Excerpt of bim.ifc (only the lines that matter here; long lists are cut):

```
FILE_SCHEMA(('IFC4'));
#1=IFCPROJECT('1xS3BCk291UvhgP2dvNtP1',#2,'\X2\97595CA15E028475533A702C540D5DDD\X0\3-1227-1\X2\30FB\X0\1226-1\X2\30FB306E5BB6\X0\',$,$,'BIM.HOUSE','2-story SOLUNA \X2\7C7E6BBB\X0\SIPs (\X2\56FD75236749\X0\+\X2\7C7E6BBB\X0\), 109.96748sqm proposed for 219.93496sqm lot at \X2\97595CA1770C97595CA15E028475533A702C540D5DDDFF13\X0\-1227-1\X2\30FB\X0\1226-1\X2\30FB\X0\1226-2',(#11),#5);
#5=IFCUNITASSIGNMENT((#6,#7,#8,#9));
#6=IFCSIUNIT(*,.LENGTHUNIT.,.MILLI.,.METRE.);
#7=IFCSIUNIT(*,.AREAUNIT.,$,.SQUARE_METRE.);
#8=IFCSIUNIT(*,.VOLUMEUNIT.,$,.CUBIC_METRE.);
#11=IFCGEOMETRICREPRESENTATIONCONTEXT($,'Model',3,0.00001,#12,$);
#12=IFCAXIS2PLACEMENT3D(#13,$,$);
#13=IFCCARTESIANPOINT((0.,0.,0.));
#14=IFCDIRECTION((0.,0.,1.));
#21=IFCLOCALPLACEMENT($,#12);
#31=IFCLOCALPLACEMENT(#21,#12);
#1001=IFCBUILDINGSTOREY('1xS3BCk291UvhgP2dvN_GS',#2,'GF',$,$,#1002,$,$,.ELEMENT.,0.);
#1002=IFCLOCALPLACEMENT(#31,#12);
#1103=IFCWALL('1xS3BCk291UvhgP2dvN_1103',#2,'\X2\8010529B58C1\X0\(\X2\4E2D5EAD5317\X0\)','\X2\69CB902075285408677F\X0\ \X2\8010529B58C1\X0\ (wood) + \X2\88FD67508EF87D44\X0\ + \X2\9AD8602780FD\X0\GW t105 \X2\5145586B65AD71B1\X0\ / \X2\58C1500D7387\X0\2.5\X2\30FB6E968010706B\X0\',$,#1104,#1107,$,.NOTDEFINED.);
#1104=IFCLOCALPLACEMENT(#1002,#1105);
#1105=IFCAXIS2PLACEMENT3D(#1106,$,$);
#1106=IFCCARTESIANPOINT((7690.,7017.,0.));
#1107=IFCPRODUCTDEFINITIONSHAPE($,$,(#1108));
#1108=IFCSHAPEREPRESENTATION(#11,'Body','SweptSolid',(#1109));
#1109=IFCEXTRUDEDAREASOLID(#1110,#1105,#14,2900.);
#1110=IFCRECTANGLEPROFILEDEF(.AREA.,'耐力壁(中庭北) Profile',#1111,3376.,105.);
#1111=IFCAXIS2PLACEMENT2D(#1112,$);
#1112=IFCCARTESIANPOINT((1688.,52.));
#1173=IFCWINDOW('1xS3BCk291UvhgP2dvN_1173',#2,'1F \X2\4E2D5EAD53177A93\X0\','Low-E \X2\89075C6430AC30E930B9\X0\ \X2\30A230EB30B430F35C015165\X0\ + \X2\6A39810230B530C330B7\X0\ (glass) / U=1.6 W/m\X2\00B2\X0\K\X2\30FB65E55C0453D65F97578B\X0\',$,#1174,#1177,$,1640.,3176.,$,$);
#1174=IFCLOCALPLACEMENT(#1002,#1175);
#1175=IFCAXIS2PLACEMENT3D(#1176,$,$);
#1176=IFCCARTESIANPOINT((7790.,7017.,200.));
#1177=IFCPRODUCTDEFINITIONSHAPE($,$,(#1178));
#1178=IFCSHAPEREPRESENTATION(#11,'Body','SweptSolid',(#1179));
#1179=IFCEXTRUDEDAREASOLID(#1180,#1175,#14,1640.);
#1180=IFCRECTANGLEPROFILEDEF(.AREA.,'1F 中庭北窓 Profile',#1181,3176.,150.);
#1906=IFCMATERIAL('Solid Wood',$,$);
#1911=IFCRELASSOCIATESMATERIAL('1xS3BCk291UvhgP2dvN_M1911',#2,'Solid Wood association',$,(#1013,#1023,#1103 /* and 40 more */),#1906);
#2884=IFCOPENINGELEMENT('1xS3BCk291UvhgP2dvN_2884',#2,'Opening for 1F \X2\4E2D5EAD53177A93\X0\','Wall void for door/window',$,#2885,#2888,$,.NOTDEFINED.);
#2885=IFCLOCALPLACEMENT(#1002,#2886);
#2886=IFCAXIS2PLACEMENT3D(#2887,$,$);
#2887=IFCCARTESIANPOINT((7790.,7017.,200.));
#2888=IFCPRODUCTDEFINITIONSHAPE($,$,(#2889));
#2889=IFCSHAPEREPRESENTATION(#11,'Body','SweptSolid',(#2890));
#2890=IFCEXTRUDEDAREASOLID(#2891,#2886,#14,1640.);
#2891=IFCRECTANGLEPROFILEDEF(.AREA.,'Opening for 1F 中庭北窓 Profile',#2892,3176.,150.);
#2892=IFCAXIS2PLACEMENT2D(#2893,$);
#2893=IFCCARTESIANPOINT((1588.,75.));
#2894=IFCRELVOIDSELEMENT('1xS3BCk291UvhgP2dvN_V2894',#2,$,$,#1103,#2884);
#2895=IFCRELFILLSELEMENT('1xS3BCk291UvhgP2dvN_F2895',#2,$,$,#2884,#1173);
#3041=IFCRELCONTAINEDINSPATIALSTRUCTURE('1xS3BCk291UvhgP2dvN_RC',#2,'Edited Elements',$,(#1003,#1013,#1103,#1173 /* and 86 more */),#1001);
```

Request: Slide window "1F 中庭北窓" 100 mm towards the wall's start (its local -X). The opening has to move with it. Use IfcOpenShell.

```python
import ifcopenshell
import ifcopenshell.api.geometry
import ifcopenshell.util.placement

model = ifcopenshell.open("bim.ifc")

window = model.by_guid("1xS3BCk291UvhgP2dvN_1173")
opening = window.FillsVoids[0].RelatingOpeningElement
wall = opening.VoidsElements[0].RelatingBuildingElement

wall_matrix = ifcopenshell.util.placement.get_local_placement(wall.ObjectPlacement)
shift = wall_matrix[:3, 0] * -100.0
before = ifcopenshell.util.placement.get_local_placement(window.ObjectPlacement)[:3, 3].copy()

# The window is not placed relative to its opening, so move both.
for product in (opening, window):
    matrix = ifcopenshell.util.placement.get_local_placement(product.ObjectPlacement)
    matrix[:3, 3] += shift
    ifcopenshell.api.geometry.edit_object_placement(model, product=product, matrix=matrix, is_si=False)

after = ifcopenshell.util.placement.get_local_placement(window.ObjectPlacement)[:3, 3]
print("window moved by", (after - before).round(3) + 0.0)

model.write("bim_updated.ifc")
```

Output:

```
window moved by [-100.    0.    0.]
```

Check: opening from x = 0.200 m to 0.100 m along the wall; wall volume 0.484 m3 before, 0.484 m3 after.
